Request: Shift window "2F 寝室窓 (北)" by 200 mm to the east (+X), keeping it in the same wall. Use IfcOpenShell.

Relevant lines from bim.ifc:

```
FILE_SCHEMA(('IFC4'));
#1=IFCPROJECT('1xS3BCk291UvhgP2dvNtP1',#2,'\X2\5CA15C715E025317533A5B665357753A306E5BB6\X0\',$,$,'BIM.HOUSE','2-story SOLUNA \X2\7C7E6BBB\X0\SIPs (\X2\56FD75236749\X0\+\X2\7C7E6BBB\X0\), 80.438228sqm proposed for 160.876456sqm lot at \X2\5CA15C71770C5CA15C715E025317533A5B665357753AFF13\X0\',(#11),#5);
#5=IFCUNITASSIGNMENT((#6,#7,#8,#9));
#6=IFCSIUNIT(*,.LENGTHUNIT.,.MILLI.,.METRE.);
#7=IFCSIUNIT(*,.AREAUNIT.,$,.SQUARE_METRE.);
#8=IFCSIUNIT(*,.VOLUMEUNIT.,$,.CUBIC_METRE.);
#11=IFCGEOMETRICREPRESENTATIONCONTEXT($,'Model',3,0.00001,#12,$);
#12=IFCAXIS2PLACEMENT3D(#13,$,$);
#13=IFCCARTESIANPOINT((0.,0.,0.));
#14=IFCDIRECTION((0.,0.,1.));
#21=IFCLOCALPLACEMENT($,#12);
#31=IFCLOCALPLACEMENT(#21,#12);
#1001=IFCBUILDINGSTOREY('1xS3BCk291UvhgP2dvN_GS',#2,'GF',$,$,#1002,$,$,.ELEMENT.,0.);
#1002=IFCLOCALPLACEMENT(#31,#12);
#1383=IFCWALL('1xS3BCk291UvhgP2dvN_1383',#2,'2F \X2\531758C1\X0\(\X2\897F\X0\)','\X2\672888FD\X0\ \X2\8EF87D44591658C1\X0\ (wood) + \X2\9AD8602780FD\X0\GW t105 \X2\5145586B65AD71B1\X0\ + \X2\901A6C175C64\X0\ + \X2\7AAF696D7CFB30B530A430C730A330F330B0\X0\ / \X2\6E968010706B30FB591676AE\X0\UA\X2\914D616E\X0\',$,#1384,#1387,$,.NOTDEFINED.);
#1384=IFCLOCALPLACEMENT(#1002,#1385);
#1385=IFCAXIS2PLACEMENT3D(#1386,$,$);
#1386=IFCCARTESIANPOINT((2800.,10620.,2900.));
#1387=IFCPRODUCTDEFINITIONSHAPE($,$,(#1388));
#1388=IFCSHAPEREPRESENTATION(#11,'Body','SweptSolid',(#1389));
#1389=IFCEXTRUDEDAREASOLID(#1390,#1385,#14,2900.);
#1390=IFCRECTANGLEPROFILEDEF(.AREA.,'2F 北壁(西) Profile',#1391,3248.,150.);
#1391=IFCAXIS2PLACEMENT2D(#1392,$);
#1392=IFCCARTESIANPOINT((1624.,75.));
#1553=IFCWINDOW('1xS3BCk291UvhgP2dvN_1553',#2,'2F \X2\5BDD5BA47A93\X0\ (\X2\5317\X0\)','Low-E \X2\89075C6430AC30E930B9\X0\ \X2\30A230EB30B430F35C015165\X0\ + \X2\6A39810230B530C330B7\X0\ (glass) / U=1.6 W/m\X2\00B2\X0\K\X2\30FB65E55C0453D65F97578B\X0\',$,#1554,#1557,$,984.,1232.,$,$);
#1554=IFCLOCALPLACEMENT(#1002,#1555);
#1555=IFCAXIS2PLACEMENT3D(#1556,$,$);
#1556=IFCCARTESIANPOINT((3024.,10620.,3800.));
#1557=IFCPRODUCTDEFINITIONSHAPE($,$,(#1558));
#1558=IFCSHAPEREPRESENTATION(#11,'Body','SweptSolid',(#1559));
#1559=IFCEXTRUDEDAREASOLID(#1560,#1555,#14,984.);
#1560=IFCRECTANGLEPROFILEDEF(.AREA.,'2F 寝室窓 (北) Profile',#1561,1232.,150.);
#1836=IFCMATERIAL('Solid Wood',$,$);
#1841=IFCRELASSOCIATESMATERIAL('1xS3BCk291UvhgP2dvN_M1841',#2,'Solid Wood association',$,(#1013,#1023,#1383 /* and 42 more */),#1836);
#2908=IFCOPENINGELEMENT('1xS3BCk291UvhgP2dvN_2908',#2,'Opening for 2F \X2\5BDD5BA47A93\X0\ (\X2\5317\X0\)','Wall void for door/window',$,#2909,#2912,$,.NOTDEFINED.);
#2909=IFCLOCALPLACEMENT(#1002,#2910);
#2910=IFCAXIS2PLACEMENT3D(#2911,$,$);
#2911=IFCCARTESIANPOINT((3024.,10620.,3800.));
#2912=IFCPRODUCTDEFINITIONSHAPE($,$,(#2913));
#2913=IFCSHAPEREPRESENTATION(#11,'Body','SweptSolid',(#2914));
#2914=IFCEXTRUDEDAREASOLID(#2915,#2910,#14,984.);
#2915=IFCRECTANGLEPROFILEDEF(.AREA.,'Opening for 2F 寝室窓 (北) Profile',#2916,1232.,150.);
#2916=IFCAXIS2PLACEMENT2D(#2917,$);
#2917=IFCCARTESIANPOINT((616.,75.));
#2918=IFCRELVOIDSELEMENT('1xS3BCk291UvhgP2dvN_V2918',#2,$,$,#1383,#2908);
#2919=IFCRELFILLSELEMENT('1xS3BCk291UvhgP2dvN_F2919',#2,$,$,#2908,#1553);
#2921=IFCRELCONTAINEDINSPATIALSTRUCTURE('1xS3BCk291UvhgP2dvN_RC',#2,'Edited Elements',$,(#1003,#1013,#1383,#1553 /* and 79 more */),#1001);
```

```python
import ifcopenshell
import ifcopenshell.api.geometry
import ifcopenshell.util.placement
import ifcopenshell.util.unit

model = ifcopenshell.open("bim.ifc")
unit_scale = ifcopenshell.util.unit.calculate_unit_scale(model)

window = model.by_guid("1xS3BCk291UvhgP2dvN_1553")
opening = window.FillsVoids[0].RelatingOpeningElement
wall = opening.VoidsElements[0].RelatingBuildingElement

wall_matrix = ifcopenshell.util.placement.get_local_placement(wall.ObjectPlacement)
shift = wall_matrix[:3, 0] * 0.2 / unit_scale
before = ifcopenshell.util.placement.get_local_placement(window.ObjectPlacement)[:3, 3].copy()

# The window is not placed relative to its opening, so move both.
for product in (opening, window):
    matrix = ifcopenshell.util.placement.get_local_placement(product.ObjectPlacement)
    matrix[:3, 3] += shift
    ifcopenshell.api.geometry.edit_object_placement(model, product=product, matrix=matrix, is_si=False)

after = ifcopenshell.util.placement.get_local_placement(window.ObjectPlacement)[:3, 3]
print("window moved by", (after - before).round(3) + 0.0)

model.write("bim_rev.ifc")
```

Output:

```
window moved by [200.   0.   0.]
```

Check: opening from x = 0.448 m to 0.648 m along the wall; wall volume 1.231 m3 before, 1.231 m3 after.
